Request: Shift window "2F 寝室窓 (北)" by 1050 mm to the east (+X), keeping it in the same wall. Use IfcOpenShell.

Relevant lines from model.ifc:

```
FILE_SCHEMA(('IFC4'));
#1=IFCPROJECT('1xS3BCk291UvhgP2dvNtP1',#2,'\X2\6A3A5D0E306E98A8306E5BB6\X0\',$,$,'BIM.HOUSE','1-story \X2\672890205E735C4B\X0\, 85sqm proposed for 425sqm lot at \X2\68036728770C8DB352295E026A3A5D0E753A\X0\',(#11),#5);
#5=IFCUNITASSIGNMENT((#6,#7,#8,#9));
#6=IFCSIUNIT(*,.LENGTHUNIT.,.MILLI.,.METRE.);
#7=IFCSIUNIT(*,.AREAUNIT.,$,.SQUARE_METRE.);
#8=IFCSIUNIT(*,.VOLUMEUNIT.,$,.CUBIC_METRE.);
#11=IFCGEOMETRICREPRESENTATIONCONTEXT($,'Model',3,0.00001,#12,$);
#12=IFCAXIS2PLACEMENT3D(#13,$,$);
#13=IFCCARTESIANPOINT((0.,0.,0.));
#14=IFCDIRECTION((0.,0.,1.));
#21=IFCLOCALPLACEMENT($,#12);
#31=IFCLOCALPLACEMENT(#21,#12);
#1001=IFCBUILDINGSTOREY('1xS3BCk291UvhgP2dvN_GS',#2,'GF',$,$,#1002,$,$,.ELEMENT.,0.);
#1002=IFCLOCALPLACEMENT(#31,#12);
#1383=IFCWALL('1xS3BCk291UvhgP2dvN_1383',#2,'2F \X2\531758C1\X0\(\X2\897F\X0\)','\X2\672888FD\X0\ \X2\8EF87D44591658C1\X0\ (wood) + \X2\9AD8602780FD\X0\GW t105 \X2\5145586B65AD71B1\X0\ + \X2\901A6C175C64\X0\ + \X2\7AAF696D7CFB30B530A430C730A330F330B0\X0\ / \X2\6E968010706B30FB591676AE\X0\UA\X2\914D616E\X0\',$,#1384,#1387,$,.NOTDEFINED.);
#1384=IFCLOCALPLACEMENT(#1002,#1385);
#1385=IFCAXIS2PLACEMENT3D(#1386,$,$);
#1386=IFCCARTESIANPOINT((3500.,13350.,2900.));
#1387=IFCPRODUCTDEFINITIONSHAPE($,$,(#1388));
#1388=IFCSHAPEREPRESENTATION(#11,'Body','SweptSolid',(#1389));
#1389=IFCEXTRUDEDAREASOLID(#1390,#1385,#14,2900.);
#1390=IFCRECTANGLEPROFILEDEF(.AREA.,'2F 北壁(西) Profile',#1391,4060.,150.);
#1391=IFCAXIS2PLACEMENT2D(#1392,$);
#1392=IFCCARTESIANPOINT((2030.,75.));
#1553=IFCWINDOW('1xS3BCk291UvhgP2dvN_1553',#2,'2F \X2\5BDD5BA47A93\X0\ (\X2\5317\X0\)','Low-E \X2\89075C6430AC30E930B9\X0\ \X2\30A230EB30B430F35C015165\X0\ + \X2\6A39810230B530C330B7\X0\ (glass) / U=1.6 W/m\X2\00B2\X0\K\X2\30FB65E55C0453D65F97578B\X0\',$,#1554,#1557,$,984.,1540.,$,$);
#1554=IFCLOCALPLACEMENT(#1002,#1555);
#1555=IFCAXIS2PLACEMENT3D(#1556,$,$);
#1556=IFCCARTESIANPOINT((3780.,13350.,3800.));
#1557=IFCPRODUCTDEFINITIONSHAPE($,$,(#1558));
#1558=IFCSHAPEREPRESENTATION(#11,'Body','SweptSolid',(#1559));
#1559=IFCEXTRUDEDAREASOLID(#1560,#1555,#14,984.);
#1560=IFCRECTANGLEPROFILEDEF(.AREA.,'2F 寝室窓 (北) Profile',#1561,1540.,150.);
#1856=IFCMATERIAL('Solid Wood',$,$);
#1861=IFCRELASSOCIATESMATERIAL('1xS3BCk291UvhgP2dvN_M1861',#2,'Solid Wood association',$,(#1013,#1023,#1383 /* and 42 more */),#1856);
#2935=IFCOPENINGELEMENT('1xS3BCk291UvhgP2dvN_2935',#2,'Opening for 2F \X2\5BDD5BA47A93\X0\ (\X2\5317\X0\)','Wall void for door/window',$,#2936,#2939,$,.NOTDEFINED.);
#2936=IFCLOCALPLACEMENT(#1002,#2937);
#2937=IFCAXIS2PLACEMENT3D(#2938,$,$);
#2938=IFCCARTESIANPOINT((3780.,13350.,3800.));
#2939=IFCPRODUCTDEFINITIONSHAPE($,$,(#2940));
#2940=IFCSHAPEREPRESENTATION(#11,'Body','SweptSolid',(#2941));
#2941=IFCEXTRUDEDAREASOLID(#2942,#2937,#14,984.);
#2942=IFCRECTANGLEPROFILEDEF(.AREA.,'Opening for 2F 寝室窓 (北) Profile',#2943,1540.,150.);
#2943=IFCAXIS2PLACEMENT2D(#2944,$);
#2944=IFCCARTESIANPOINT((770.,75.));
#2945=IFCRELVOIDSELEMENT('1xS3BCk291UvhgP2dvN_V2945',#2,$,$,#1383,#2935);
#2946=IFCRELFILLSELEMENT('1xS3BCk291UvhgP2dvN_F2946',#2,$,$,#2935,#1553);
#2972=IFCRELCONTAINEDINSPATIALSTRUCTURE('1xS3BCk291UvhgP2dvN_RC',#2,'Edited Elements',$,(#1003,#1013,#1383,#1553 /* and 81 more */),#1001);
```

```python
import ifcopenshell
import ifcopenshell.api.geometry
import ifcopenshell.util.placement
import ifcopenshell.util.unit

model = ifcopenshell.open("model.ifc")
unit_scale = ifcopenshell.util.unit.calculate_unit_scale(model)

window = model.by_guid("1xS3BCk291UvhgP2dvN_1553")
opening = window.FillsVoids[0].RelatingOpeningElement
wall = opening.VoidsElements[0].RelatingBuildingElement

wall_matrix = ifcopenshell.util.placement.get_local_placement(wall.ObjectPlacement)
shift = wall_matrix[:3, 0] * 1.05 / unit_scale
before = ifcopenshell.util.placement.get_local_placement(window.ObjectPlacement)[:3, 3].copy()

# The window is not placed relative to its opening, so move both.
for product in (opening, window):
    matrix = ifcopenshell.util.placement.get_local_placement(product.ObjectPlacement)
    matrix[:3, 3] += shift
    ifcopenshell.api.geometry.edit_object_placement(model, product=product, matrix=matrix, is_si=False)

after = ifcopenshell.util.placement.get_local_placement(window.ObjectPlacement)[:3, 3]
print("window moved by", (after - before).round(3) + 0.0)

model.write("model_v2.ifc")
```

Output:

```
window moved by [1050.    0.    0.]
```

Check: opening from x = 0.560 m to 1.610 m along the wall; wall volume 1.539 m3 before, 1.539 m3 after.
